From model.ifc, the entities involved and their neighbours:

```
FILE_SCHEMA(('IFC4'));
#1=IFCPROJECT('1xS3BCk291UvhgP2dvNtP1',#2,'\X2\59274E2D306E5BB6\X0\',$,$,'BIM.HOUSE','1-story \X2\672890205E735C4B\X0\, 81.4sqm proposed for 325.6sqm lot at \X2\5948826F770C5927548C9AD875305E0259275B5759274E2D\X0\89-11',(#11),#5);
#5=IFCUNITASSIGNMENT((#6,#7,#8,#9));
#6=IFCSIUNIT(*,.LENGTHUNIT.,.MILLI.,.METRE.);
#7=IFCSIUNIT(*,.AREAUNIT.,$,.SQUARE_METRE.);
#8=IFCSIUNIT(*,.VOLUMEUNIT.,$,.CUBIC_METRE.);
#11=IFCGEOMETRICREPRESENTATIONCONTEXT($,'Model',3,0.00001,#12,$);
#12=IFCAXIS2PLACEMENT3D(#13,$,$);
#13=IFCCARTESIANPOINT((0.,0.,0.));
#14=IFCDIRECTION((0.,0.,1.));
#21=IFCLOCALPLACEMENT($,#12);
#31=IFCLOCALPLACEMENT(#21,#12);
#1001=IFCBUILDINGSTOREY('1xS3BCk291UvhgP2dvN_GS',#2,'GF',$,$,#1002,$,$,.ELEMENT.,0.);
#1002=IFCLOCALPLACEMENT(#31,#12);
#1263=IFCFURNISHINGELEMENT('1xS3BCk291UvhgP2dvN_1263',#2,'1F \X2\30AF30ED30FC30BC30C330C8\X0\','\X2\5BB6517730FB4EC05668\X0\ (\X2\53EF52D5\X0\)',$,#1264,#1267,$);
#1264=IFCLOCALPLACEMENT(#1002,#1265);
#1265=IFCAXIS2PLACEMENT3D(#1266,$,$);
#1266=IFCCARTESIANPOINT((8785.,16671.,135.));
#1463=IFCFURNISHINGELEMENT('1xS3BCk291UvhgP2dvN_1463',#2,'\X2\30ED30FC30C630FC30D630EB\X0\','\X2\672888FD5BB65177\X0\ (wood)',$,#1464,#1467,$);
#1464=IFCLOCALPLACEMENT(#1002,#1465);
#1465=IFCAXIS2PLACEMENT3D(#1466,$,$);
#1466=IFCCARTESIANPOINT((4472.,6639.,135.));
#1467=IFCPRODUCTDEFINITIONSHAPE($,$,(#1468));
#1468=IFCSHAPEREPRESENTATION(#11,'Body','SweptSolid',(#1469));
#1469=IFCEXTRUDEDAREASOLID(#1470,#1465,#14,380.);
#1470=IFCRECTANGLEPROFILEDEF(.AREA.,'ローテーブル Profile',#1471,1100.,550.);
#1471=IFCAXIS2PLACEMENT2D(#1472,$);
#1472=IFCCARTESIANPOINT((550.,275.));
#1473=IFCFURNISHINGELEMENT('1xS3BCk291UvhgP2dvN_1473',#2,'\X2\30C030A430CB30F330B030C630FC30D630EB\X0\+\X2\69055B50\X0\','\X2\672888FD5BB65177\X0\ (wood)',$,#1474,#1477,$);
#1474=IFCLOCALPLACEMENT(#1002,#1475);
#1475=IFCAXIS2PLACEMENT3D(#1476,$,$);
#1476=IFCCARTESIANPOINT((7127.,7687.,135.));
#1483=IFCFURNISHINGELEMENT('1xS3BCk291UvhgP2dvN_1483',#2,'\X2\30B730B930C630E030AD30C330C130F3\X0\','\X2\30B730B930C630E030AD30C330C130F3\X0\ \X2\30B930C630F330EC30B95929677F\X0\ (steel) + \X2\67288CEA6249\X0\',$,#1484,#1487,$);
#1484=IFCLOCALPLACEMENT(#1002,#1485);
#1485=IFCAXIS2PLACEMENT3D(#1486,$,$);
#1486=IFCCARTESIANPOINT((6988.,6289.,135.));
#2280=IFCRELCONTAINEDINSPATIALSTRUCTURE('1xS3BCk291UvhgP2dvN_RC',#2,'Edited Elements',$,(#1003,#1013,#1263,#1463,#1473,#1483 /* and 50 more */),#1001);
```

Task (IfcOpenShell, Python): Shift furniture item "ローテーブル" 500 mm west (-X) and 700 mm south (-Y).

```python
import ifcopenshell
import ifcopenshell.api.geometry
import ifcopenshell.util.placement

model = ifcopenshell.open("model.ifc")

item = model.by_guid("1xS3BCk291UvhgP2dvN_1463")
matrix = ifcopenshell.util.placement.get_local_placement(item.ObjectPlacement)
matrix[0, 3] -= 500.0
matrix[1, 3] -= 700.0
ifcopenshell.api.geometry.edit_object_placement(model, product=item, matrix=matrix, is_si=False)

print(ifcopenshell.util.placement.get_local_placement(item.ObjectPlacement).round(3) + 0.0)

model.write("model_v2.ifc")
```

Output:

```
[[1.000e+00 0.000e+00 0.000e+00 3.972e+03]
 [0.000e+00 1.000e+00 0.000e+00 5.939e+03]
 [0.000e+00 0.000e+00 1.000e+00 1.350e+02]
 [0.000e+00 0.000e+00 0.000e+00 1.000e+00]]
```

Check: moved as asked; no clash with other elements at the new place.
